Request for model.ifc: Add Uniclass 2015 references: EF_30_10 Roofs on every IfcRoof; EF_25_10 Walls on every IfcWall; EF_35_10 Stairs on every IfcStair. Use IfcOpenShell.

First a look at what the model holds.

```python
import ifcopenshell

model = ifcopenshell.open("model.ifc")
print(model.schema)
print("classifications:", [c.Name for c in model.by_type("IfcClassification")])
for ifc_class in ("IfcDoor", "IfcRoof", "IfcStair", "IfcWall", "IfcWindow"):
    print(ifc_class, len(model.by_type(ifc_class)))
```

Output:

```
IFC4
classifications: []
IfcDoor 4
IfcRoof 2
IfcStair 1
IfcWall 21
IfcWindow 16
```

```python
import ifcopenshell
import ifcopenshell.api.classification

model = ifcopenshell.open("model.ifc")

system = ifcopenshell.api.classification.add_classification(model, classification="Uniclass 2015")

codes = {
    "IfcRoof": ("EF_30_10", "Roofs"),
    "IfcWall": ("EF_25_10", "Walls"),
    "IfcStair": ("EF_35_10", "Stairs"),
}
for ifc_class, (code, name) in codes.items():
    products = model.by_type(ifc_class)
    ifcopenshell.api.classification.add_reference(
        model, products=products, classification=system, identification=code, name=name
    )
    print(code, len(products))

model.write("model_updated.ifc")
```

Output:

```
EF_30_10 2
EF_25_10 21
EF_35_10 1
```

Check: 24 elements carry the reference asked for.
